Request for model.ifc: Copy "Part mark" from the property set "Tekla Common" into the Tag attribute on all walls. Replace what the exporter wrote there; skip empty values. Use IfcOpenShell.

First a look at what the model holds.

```python
import ifcopenshell
import ifcopenshell.util.element

model = ifcopenshell.open("model.ifc")
print(model.schema)
walls = model.by_type("IfcWall")
print(len(walls), "walls")
for e in walls[:8]:
    source = ifcopenshell.util.element.get_pset(e, "Tekla Common", "Part mark")
    target = e.Tag
    print(e.id(), repr(source), repr(target), sep=" | ")
```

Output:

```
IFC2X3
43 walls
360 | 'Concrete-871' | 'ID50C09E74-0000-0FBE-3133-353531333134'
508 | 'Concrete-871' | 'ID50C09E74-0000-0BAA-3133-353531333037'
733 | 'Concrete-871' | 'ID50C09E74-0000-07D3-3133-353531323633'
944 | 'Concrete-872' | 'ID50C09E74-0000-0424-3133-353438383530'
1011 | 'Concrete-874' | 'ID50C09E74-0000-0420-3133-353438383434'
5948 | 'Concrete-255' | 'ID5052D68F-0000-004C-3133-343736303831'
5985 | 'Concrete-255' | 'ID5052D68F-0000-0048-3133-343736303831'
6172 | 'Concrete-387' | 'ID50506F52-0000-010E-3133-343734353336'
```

```python
import ifcopenshell
import ifcopenshell.util.element

model = ifcopenshell.open("model.ifc")

count = 0
for e in model.by_type("IfcWall"):
    value = ifcopenshell.util.element.get_pset(e, "Tekla Common", "Part mark")
    current = e.Tag
    if not value or not value.strip() or current == value:
        continue
    e.Tag = value
    count += 1

print(count, "walls updated")

model.write("model-out.ifc")
```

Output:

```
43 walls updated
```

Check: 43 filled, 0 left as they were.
